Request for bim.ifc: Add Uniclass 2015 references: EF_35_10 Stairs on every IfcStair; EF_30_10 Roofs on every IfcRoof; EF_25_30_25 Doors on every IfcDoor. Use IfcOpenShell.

First a look at what the model holds.

```python
import ifcopenshell

model = ifcopenshell.open("bim.ifc")
print(model.schema)
print("classifications:", [c.Name for c in model.by_type("IfcClassification")])
for ifc_class in ("IfcDoor", "IfcRoof", "IfcStair", "IfcWall", "IfcWindow"):
    print(ifc_class, len(model.by_type(ifc_class)))
```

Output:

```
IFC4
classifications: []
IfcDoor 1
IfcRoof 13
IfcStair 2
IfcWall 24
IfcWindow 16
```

```python
import ifcopenshell
import ifcopenshell.api.classification

model = ifcopenshell.open("bim.ifc")

system = ifcopenshell.api.classification.add_classification(model, classification="Uniclass 2015")

codes = {
    "IfcStair": ("EF_35_10", "Stairs"),
    "IfcRoof": ("EF_30_10", "Roofs"),
    "IfcDoor": ("EF_25_30_25", "Doors"),
}
for ifc_class, (code, name) in codes.items():
    products = model.by_type(ifc_class)
    ifcopenshell.api.classification.add_reference(
        model, products=products, classification=system, identification=code, name=name
    )
    print(code, len(products))

model.write("bim_edited.ifc")
```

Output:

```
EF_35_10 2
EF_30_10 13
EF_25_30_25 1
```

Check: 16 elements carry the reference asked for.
